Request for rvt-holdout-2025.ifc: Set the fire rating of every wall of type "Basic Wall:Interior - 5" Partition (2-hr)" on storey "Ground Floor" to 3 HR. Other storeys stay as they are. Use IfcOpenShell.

First a look at what the model holds.

```python
import ifcopenshell
import ifcopenshell.util.element

model = ifcopenshell.open("rvt-holdout-2025.ifc")
print(model.schema)
storey = next(s for s in model.by_type("IfcBuildingStorey") if s.Name == "Ground Floor")
walls = [e for e in ifcopenshell.util.element.get_decomposition(storey) if e.is_a("IfcWall")]
seen = {}
for e in walls:
    element_type = ifcopenshell.util.element.get_type(e)
    key = (element_type.Name if element_type != e and element_type else None, ifcopenshell.util.element.get_pset(e, "Pset_WallCommon", "FireRating"))
    seen[key] = seen.get(key, 0) + 1
for (name, value), count in sorted(seen.items(), key=str):
    print(count, "x", name, "|", value)
```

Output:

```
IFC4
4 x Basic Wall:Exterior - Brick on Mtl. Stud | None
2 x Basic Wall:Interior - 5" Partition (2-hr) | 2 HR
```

```python
import ifcopenshell
import ifcopenshell.api.pset
import ifcopenshell.util.element

model = ifcopenshell.open("rvt-holdout-2025.ifc")

storey = next(s for s in model.by_type("IfcBuildingStorey") if s.Name == "Ground Floor")
walls = [e for e in ifcopenshell.util.element.get_decomposition(storey) if e.is_a("IfcWall")]

count = 0
for e in walls:
    element_type = ifcopenshell.util.element.get_type(e)
    if element_type in (None, e) or element_type.Name != 'Basic Wall:Interior - 5" Partition (2-hr)':
        continue
    # add_pset returns the element's existing set when there is one.
    pset = ifcopenshell.api.pset.add_pset(model, product=e, name="Pset_WallCommon")
    ifcopenshell.api.pset.edit_pset(model, pset=pset, properties={"FireRating": "3 HR"})
    count += 1

print(count, "walls updated")

model.write("rvt-holdout-2025_rev.ifc")
```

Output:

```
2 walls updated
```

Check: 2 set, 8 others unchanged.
